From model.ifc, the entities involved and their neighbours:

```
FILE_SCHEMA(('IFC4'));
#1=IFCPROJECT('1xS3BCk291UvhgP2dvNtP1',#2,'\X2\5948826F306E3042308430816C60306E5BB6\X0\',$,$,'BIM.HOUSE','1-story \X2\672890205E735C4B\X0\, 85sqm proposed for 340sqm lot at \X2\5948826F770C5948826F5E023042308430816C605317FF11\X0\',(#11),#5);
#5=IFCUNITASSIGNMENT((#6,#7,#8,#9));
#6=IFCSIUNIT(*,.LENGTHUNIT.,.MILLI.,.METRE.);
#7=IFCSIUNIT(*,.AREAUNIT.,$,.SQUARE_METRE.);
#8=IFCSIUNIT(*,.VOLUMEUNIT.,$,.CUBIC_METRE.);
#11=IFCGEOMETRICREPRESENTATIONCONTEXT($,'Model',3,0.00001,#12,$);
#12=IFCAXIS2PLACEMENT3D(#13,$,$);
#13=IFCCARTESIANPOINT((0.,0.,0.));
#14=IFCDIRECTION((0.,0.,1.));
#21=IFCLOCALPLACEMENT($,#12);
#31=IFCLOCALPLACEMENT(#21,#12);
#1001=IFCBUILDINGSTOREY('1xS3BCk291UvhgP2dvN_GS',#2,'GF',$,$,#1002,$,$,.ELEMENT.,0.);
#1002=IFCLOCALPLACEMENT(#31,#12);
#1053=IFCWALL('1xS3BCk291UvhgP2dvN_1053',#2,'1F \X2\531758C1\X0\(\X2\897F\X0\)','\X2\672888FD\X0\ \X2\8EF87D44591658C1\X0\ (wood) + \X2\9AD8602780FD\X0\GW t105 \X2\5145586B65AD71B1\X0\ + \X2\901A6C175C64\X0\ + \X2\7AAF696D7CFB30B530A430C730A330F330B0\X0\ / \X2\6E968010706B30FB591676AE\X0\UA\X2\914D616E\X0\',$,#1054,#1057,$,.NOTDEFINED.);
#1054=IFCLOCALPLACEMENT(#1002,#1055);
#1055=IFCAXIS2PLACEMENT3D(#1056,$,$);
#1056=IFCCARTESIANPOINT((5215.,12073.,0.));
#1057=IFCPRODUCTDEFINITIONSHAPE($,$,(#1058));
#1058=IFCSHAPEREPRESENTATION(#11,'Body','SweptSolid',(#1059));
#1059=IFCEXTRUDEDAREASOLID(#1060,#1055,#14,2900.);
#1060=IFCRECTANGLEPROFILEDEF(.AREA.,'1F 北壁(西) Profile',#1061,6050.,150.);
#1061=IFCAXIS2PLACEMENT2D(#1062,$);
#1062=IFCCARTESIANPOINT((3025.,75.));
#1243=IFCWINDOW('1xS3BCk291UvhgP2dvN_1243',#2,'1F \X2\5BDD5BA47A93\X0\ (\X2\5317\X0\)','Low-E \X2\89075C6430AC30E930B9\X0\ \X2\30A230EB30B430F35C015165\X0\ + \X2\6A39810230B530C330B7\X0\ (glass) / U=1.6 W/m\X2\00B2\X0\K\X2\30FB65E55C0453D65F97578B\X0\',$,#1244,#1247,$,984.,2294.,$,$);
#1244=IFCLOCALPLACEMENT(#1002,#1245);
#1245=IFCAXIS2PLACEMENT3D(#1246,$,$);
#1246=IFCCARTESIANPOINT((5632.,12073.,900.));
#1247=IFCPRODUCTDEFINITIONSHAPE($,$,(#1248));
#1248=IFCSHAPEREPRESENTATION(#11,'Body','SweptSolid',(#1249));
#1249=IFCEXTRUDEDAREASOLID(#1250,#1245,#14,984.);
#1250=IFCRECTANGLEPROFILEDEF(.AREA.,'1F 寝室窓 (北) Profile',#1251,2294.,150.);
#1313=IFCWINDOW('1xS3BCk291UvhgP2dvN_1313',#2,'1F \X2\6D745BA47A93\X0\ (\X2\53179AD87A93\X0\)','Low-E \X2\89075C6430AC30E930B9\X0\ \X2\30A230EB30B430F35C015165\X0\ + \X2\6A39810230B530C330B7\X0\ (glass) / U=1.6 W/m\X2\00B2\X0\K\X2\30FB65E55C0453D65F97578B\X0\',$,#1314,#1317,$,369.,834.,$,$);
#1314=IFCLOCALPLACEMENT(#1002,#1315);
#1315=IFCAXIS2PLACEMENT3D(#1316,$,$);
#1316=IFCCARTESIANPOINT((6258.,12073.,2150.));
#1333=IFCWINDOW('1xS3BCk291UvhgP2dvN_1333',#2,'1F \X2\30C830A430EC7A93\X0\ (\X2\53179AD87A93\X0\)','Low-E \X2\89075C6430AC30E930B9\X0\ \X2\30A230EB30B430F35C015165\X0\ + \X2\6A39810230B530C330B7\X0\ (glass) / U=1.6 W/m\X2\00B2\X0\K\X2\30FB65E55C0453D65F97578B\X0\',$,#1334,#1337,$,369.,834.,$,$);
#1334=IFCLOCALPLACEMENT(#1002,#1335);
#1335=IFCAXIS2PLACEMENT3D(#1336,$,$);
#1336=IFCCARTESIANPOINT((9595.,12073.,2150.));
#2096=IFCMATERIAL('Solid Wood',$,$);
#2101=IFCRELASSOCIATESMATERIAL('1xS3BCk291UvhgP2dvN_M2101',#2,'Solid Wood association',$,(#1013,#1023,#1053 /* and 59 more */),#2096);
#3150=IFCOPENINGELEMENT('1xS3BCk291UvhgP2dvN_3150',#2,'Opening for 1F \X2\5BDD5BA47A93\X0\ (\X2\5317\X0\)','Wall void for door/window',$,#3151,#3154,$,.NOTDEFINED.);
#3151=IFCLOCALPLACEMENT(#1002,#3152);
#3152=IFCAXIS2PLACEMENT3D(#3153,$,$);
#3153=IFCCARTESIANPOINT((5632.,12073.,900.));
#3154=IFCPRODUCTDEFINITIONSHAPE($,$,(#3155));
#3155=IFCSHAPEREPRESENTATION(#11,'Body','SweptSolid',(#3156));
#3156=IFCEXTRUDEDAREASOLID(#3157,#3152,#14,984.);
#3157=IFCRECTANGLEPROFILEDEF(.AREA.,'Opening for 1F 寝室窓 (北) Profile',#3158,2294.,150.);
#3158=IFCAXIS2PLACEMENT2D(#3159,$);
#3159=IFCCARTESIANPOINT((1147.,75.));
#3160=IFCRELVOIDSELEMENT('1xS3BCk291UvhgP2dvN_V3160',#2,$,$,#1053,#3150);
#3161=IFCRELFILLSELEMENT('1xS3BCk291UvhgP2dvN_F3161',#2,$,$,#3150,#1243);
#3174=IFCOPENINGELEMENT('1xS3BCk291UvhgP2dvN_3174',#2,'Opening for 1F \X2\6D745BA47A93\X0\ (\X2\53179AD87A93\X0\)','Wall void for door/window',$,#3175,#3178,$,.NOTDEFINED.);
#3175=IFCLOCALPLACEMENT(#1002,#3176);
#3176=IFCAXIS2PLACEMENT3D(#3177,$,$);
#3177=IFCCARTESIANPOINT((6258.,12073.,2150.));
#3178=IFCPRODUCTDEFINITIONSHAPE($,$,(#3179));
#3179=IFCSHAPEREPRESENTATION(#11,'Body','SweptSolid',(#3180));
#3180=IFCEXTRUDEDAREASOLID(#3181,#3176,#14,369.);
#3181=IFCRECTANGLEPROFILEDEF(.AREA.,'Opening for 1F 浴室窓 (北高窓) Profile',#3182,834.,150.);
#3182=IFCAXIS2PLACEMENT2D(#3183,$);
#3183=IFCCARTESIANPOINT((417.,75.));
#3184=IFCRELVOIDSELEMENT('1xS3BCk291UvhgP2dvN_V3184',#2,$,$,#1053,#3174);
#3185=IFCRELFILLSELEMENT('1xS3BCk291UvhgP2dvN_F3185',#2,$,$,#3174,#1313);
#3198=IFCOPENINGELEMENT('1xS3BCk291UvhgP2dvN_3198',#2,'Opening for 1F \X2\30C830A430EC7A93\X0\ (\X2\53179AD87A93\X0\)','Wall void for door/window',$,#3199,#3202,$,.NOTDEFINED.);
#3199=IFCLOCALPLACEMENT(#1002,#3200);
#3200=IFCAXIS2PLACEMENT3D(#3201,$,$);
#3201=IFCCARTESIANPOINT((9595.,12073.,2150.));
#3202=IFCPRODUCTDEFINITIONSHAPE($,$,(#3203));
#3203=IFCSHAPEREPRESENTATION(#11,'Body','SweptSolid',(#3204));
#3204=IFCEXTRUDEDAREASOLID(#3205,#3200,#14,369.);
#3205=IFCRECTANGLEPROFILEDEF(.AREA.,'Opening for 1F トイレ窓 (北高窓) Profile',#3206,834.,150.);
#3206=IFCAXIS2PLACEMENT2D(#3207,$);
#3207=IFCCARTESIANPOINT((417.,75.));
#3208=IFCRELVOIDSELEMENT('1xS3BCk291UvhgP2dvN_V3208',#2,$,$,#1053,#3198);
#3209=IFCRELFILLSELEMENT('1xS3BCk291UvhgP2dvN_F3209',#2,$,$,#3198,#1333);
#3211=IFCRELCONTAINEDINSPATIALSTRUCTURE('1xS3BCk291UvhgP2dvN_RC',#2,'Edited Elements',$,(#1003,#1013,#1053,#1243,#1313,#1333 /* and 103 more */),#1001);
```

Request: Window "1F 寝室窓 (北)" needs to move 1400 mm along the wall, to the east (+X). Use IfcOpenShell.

```python
import ifcopenshell
import ifcopenshell.api.geometry
import ifcopenshell.util.placement
import ifcopenshell.util.unit

model = ifcopenshell.open("model.ifc")
unit_scale = ifcopenshell.util.unit.calculate_unit_scale(model)

window = model.by_guid("1xS3BCk291UvhgP2dvN_1243")
opening = window.FillsVoids[0].RelatingOpeningElement
wall = opening.VoidsElements[0].RelatingBuildingElement

wall_matrix = ifcopenshell.util.placement.get_local_placement(wall.ObjectPlacement)
shift = wall_matrix[:3, 0] * 1.4 / unit_scale
before = ifcopenshell.util.placement.get_local_placement(window.ObjectPlacement)[:3, 3].copy()

# The window is not placed relative to its opening, so move both.
for product in (opening, window):
    matrix = ifcopenshell.util.placement.get_local_placement(product.ObjectPlacement)
    matrix[:3, 3] += shift
    ifcopenshell.api.geometry.edit_object_placement(model, product=product, matrix=matrix, is_si=False)

after = ifcopenshell.util.placement.get_local_placement(window.ObjectPlacement)[:3, 3]
print("window moved by", (after - before).round(3) + 0.0)

model.write("model_rev.ifc")
```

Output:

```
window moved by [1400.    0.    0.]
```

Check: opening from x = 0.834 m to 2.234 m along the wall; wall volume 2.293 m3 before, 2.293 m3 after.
